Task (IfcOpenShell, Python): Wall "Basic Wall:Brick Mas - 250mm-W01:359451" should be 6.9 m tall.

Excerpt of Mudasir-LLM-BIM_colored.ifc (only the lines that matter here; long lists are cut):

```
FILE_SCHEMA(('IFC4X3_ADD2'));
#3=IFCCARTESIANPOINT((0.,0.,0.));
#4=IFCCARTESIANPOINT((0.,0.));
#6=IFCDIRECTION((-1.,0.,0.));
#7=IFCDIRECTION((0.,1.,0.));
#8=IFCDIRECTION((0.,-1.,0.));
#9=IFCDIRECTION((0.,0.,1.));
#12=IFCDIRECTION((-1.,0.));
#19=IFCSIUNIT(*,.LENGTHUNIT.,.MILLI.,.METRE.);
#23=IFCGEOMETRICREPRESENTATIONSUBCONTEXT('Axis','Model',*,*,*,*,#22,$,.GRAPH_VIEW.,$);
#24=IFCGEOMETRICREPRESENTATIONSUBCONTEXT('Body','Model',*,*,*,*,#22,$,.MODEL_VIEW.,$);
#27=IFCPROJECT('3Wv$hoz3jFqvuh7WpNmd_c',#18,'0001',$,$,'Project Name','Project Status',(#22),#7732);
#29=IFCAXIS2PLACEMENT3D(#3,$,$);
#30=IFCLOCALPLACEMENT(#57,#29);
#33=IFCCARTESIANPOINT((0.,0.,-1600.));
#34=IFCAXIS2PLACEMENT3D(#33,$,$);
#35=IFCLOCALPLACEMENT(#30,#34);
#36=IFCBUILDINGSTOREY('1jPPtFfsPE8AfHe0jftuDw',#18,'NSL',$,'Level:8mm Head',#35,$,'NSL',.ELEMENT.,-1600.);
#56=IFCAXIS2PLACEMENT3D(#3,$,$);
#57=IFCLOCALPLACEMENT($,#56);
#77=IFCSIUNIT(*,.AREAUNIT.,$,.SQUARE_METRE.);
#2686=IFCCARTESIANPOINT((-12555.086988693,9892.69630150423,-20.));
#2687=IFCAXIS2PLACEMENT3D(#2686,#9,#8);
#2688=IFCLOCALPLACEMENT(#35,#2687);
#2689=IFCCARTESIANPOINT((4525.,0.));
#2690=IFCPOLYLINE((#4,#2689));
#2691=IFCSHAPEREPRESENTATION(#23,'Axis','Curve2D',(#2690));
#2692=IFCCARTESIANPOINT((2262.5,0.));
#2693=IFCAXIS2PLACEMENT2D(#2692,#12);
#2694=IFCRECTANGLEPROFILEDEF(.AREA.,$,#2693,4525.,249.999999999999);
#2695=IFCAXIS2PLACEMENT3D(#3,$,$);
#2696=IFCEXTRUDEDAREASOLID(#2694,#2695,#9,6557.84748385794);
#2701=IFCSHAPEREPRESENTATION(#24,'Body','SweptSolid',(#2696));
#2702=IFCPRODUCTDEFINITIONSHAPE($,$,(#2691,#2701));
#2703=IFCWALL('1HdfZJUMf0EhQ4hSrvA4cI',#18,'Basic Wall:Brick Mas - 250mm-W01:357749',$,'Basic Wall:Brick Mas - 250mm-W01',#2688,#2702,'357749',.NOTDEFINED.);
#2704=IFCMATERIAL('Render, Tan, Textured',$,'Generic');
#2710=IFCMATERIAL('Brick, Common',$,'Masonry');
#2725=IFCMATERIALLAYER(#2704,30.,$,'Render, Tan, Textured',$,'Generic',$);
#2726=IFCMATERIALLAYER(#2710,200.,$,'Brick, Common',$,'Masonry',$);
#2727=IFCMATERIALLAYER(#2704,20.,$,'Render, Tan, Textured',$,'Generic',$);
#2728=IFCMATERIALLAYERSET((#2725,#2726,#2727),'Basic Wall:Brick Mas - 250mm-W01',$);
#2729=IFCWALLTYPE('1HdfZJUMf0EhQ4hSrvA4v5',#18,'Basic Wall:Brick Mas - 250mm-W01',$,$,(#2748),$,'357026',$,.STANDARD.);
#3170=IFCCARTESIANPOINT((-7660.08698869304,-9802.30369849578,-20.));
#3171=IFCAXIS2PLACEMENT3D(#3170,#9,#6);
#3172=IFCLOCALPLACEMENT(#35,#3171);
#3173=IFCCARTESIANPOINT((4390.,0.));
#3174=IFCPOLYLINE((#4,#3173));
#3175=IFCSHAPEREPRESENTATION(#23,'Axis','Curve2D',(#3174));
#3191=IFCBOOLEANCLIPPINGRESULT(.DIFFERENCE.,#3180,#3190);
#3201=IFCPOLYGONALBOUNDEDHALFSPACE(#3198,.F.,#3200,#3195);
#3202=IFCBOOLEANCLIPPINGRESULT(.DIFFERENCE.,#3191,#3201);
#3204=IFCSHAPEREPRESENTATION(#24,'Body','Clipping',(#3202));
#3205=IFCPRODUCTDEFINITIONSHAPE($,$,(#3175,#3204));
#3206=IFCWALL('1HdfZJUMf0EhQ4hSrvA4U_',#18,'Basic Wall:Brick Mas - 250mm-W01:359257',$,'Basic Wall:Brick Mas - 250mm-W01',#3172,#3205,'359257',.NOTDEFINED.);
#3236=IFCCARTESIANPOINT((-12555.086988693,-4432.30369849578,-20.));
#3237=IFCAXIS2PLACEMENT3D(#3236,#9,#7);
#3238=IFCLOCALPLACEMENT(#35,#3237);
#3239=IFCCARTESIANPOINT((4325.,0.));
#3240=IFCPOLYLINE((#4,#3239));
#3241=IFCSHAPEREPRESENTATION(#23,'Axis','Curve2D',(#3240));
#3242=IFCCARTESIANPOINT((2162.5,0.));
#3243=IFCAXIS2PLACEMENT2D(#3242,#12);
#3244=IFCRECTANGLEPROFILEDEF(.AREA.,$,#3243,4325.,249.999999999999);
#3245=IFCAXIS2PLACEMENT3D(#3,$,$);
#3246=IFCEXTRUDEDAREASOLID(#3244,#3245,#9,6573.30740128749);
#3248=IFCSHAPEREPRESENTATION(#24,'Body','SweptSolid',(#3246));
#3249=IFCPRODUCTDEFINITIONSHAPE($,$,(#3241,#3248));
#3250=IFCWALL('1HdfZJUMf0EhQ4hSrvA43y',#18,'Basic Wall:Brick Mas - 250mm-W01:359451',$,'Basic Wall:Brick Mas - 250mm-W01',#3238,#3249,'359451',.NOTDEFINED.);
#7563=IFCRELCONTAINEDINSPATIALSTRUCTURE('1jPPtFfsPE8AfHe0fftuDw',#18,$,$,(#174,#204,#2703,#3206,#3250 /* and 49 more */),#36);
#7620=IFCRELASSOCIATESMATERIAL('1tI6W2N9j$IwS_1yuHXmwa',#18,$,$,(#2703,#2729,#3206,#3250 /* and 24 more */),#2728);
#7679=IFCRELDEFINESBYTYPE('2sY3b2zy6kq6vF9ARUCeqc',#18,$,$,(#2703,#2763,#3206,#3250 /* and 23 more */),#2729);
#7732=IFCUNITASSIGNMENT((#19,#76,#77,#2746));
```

```python
import ifcopenshell
import ifcopenshell.geom
import ifcopenshell.util.representation
import ifcopenshell.util.shape
import ifcopenshell.util.unit

model = ifcopenshell.open("Mudasir-LLM-BIM_colored.ifc")
unit_scale = ifcopenshell.util.unit.calculate_unit_scale(model)
settings = ifcopenshell.geom.settings()


def volume(element):
    """Net volume in cubic metres, openings subtracted."""
    shape = ifcopenshell.geom.create_shape(settings, element)
    return ifcopenshell.util.shape.get_volume(shape.geometry)


wall = model.by_id(3250)
before = volume(wall)

body = ifcopenshell.util.representation.get_representation(wall, "Model", "Body")
solid = body.Items[0]
old_height = solid.Depth
solid.Depth = 6.9 / unit_scale
after = volume(wall)

print(f"height {old_height:g} -> {solid.Depth:g}, volume {before:.3f} -> {after:.3f} m3")

model.write("Mudasir-LLM-BIM_colored_rev.ifc")
```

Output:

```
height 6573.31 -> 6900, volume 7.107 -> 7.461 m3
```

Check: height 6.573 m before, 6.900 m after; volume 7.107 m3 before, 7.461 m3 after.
